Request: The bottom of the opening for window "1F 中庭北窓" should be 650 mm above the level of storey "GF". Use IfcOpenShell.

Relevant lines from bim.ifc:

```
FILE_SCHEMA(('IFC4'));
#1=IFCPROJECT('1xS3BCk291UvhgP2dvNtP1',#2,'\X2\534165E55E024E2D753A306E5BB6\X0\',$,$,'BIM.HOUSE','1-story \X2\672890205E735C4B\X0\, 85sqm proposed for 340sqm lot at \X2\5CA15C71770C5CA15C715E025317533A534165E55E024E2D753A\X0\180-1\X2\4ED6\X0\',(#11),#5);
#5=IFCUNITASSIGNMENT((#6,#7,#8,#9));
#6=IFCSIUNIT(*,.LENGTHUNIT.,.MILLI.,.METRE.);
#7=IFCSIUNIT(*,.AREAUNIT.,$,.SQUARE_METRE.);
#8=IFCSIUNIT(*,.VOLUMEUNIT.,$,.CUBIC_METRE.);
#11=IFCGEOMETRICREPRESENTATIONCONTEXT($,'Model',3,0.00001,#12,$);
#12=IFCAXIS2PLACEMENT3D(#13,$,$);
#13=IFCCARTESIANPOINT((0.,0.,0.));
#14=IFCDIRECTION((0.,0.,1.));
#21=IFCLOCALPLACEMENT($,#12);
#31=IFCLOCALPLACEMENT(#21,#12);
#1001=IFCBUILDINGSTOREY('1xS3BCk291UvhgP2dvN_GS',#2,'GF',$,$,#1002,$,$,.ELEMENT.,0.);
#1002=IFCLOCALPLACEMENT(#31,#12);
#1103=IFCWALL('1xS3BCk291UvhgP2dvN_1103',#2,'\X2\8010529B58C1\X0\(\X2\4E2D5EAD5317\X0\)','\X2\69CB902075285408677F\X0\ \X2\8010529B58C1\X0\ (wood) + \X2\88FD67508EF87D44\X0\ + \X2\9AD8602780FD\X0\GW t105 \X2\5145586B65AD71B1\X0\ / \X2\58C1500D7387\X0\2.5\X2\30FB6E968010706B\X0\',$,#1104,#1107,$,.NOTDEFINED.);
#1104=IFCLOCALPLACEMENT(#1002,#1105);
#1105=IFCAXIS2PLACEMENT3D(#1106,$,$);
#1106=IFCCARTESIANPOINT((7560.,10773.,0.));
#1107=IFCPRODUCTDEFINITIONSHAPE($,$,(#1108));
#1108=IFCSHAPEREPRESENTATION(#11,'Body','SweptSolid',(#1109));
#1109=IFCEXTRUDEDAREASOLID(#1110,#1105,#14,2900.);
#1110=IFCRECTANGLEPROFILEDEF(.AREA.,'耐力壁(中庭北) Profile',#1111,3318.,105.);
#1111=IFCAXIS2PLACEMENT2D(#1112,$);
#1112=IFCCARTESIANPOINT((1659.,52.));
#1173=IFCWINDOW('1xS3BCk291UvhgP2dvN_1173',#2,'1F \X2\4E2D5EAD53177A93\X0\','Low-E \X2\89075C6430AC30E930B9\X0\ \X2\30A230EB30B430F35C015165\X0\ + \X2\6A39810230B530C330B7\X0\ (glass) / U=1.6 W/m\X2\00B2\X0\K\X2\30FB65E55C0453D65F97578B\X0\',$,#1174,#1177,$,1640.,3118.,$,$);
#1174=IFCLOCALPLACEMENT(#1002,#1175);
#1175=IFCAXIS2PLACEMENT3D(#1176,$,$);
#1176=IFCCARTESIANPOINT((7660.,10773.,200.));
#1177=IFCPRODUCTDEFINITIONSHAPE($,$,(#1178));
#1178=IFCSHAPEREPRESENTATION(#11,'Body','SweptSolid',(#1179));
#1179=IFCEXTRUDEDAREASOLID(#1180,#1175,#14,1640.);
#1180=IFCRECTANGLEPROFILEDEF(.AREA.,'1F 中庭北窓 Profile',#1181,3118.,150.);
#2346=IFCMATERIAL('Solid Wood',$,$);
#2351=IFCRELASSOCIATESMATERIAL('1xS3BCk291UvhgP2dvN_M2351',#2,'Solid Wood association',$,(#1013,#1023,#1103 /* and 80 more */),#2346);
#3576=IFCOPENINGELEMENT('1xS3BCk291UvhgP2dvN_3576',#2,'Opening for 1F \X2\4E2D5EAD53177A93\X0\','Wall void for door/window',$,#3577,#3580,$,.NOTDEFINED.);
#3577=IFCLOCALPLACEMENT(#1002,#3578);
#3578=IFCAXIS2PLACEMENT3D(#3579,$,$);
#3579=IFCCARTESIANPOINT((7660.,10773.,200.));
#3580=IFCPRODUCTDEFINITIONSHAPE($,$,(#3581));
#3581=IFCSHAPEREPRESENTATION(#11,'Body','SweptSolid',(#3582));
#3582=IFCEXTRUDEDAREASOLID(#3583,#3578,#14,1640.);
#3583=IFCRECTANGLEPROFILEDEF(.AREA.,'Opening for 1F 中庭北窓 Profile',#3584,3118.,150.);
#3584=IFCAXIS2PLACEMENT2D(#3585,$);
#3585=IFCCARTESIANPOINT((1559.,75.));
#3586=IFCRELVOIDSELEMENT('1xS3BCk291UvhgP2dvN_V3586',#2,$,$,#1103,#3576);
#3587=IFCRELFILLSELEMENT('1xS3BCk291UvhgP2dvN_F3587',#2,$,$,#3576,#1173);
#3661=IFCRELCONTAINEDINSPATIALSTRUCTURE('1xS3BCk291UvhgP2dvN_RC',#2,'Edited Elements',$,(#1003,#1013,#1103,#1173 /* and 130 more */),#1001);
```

```python
import numpy as np
import ifcopenshell
import ifcopenshell.api.geometry
import ifcopenshell.geom
import ifcopenshell.util.element
import ifcopenshell.util.placement
import ifcopenshell.util.shape
import ifcopenshell.util.unit

model = ifcopenshell.open("bim.ifc")
unit_scale = ifcopenshell.util.unit.calculate_unit_scale(model)

window = model.by_guid("1xS3BCk291UvhgP2dvN_1173")
opening = window.FillsVoids[0].RelatingOpeningElement
storey = ifcopenshell.util.element.get_container(window, ifc_class="IfcBuildingStorey")
level = ifcopenshell.util.placement.get_local_placement(storey.ObjectPlacement)[2, 3]

# The opening's origin need not be at the sill, so measure its lowest point.
shape = ifcopenshell.geom.create_shape(ifcopenshell.geom.settings(), opening)
bottom = ifcopenshell.util.shape.get_shape_bottom_elevation(shape, shape.geometry) / unit_scale
dz = level + 650.0 - bottom

shift = np.array([0.0, 0.0, dz])
# The window is not placed relative to its opening, so move both.
for product in (opening, window):
    matrix = ifcopenshell.util.placement.get_local_placement(product.ObjectPlacement)
    matrix[:3, 3] += shift
    ifcopenshell.api.geometry.edit_object_placement(model, product=product, matrix=matrix, is_si=False)

print(f"moved by {dz * unit_scale:+.3f} m")

model.write("bim-out.ifc")
```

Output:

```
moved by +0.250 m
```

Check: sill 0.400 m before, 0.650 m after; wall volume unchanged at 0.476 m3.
